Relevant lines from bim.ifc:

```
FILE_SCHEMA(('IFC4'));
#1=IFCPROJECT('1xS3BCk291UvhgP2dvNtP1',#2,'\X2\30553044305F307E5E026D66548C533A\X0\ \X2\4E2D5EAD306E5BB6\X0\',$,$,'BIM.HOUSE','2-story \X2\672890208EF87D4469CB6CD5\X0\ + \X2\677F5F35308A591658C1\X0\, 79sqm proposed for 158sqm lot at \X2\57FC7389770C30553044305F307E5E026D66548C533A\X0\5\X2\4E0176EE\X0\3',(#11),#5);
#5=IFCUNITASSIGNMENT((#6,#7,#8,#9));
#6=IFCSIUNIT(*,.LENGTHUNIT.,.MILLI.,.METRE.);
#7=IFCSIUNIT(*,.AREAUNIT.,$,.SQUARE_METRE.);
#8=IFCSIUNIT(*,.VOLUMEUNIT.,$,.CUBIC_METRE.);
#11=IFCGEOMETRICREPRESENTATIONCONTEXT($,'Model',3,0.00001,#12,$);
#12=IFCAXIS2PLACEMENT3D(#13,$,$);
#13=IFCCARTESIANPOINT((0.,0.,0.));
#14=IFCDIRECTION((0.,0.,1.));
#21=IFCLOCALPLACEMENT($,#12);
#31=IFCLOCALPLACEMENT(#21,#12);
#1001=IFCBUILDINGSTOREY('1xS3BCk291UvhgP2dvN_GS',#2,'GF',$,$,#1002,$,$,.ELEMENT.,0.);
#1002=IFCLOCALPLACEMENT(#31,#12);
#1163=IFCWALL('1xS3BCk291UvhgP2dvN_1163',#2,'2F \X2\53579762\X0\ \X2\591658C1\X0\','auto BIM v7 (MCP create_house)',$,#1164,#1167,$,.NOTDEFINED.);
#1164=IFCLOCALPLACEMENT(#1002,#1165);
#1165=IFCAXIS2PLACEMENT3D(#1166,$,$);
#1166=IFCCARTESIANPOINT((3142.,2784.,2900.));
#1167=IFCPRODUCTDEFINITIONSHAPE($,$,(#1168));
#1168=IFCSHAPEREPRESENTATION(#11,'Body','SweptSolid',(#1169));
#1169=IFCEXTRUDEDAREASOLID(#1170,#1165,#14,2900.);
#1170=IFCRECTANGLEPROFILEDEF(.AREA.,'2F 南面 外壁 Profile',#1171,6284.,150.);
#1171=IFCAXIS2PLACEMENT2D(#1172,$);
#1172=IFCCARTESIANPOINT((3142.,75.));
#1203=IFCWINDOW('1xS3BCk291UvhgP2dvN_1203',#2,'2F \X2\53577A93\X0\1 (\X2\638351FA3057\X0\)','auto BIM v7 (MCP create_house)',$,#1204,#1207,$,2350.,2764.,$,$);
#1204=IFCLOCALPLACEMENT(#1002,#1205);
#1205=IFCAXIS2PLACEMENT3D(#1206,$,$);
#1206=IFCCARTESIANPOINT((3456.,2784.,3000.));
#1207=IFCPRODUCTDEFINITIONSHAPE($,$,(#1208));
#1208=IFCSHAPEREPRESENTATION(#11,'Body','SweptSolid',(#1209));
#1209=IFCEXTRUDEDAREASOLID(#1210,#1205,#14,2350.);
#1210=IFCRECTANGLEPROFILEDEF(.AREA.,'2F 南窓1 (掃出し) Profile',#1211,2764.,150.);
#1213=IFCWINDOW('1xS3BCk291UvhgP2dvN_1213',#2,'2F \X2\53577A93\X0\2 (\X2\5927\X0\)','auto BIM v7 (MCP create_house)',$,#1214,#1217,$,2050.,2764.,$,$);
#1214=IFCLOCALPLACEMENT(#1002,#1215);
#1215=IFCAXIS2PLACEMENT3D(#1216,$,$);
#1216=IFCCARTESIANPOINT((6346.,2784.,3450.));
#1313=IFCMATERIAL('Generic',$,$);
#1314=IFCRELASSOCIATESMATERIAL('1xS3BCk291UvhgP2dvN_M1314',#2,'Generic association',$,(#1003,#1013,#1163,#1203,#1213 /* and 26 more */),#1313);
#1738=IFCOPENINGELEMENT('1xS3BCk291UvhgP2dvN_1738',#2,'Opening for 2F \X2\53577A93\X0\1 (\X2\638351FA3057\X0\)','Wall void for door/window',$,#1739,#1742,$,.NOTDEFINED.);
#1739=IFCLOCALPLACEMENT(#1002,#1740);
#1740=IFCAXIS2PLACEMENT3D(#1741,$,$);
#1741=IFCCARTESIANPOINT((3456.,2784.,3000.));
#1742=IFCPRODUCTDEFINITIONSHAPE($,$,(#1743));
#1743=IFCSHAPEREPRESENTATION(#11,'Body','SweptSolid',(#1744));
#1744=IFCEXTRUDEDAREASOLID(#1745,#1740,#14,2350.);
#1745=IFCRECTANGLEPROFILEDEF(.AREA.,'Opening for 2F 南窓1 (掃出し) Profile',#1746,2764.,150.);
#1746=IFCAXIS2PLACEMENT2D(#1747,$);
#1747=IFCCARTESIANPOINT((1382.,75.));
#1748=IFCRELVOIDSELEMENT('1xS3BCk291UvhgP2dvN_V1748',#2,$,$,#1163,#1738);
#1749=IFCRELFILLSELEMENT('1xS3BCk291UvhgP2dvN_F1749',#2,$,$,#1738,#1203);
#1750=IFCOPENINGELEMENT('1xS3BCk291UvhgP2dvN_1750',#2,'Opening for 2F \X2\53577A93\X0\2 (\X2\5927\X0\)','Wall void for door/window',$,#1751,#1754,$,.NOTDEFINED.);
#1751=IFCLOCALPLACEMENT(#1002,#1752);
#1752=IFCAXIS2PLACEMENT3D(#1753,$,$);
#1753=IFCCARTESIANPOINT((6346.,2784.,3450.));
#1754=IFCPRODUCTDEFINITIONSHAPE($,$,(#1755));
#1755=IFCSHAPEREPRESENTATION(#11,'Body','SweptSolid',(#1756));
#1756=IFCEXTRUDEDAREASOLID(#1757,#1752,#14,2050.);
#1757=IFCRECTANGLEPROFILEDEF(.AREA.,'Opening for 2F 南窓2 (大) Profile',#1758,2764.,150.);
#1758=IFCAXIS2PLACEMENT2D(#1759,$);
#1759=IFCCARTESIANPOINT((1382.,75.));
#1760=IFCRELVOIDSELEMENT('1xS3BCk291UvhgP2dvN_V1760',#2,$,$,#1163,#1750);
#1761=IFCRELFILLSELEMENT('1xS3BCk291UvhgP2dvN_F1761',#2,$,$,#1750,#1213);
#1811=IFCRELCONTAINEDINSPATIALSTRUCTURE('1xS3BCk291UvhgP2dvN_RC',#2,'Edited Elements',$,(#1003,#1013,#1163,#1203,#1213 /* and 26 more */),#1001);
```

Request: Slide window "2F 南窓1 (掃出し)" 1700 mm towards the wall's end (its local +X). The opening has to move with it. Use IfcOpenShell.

```python
import ifcopenshell
import ifcopenshell.api.geometry
import ifcopenshell.util.placement
import ifcopenshell.util.unit

model = ifcopenshell.open("bim.ifc")
unit_scale = ifcopenshell.util.unit.calculate_unit_scale(model)

window = model.by_id(1203)
opening = window.FillsVoids[0].RelatingOpeningElement
wall = opening.VoidsElements[0].RelatingBuildingElement

wall_matrix = ifcopenshell.util.placement.get_local_placement(wall.ObjectPlacement)
shift = wall_matrix[:3, 0] * 1.7 / unit_scale
before = ifcopenshell.util.placement.get_local_placement(window.ObjectPlacement)[:3, 3].copy()

# The window is not placed relative to its opening, so move both.
for product in (opening, window):
    matrix = ifcopenshell.util.placement.get_local_placement(product.ObjectPlacement)
    matrix[:3, 3] += shift
    ifcopenshell.api.geometry.edit_object_placement(model, product=product, matrix=matrix, is_si=False)

after = ifcopenshell.util.placement.get_local_placement(window.ObjectPlacement)[:3, 3]
print("window moved by", (after - before).round(3) + 0.0)

model.write("bim_edited.ifc")
```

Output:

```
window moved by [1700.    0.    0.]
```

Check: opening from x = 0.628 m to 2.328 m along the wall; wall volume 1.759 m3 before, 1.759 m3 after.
